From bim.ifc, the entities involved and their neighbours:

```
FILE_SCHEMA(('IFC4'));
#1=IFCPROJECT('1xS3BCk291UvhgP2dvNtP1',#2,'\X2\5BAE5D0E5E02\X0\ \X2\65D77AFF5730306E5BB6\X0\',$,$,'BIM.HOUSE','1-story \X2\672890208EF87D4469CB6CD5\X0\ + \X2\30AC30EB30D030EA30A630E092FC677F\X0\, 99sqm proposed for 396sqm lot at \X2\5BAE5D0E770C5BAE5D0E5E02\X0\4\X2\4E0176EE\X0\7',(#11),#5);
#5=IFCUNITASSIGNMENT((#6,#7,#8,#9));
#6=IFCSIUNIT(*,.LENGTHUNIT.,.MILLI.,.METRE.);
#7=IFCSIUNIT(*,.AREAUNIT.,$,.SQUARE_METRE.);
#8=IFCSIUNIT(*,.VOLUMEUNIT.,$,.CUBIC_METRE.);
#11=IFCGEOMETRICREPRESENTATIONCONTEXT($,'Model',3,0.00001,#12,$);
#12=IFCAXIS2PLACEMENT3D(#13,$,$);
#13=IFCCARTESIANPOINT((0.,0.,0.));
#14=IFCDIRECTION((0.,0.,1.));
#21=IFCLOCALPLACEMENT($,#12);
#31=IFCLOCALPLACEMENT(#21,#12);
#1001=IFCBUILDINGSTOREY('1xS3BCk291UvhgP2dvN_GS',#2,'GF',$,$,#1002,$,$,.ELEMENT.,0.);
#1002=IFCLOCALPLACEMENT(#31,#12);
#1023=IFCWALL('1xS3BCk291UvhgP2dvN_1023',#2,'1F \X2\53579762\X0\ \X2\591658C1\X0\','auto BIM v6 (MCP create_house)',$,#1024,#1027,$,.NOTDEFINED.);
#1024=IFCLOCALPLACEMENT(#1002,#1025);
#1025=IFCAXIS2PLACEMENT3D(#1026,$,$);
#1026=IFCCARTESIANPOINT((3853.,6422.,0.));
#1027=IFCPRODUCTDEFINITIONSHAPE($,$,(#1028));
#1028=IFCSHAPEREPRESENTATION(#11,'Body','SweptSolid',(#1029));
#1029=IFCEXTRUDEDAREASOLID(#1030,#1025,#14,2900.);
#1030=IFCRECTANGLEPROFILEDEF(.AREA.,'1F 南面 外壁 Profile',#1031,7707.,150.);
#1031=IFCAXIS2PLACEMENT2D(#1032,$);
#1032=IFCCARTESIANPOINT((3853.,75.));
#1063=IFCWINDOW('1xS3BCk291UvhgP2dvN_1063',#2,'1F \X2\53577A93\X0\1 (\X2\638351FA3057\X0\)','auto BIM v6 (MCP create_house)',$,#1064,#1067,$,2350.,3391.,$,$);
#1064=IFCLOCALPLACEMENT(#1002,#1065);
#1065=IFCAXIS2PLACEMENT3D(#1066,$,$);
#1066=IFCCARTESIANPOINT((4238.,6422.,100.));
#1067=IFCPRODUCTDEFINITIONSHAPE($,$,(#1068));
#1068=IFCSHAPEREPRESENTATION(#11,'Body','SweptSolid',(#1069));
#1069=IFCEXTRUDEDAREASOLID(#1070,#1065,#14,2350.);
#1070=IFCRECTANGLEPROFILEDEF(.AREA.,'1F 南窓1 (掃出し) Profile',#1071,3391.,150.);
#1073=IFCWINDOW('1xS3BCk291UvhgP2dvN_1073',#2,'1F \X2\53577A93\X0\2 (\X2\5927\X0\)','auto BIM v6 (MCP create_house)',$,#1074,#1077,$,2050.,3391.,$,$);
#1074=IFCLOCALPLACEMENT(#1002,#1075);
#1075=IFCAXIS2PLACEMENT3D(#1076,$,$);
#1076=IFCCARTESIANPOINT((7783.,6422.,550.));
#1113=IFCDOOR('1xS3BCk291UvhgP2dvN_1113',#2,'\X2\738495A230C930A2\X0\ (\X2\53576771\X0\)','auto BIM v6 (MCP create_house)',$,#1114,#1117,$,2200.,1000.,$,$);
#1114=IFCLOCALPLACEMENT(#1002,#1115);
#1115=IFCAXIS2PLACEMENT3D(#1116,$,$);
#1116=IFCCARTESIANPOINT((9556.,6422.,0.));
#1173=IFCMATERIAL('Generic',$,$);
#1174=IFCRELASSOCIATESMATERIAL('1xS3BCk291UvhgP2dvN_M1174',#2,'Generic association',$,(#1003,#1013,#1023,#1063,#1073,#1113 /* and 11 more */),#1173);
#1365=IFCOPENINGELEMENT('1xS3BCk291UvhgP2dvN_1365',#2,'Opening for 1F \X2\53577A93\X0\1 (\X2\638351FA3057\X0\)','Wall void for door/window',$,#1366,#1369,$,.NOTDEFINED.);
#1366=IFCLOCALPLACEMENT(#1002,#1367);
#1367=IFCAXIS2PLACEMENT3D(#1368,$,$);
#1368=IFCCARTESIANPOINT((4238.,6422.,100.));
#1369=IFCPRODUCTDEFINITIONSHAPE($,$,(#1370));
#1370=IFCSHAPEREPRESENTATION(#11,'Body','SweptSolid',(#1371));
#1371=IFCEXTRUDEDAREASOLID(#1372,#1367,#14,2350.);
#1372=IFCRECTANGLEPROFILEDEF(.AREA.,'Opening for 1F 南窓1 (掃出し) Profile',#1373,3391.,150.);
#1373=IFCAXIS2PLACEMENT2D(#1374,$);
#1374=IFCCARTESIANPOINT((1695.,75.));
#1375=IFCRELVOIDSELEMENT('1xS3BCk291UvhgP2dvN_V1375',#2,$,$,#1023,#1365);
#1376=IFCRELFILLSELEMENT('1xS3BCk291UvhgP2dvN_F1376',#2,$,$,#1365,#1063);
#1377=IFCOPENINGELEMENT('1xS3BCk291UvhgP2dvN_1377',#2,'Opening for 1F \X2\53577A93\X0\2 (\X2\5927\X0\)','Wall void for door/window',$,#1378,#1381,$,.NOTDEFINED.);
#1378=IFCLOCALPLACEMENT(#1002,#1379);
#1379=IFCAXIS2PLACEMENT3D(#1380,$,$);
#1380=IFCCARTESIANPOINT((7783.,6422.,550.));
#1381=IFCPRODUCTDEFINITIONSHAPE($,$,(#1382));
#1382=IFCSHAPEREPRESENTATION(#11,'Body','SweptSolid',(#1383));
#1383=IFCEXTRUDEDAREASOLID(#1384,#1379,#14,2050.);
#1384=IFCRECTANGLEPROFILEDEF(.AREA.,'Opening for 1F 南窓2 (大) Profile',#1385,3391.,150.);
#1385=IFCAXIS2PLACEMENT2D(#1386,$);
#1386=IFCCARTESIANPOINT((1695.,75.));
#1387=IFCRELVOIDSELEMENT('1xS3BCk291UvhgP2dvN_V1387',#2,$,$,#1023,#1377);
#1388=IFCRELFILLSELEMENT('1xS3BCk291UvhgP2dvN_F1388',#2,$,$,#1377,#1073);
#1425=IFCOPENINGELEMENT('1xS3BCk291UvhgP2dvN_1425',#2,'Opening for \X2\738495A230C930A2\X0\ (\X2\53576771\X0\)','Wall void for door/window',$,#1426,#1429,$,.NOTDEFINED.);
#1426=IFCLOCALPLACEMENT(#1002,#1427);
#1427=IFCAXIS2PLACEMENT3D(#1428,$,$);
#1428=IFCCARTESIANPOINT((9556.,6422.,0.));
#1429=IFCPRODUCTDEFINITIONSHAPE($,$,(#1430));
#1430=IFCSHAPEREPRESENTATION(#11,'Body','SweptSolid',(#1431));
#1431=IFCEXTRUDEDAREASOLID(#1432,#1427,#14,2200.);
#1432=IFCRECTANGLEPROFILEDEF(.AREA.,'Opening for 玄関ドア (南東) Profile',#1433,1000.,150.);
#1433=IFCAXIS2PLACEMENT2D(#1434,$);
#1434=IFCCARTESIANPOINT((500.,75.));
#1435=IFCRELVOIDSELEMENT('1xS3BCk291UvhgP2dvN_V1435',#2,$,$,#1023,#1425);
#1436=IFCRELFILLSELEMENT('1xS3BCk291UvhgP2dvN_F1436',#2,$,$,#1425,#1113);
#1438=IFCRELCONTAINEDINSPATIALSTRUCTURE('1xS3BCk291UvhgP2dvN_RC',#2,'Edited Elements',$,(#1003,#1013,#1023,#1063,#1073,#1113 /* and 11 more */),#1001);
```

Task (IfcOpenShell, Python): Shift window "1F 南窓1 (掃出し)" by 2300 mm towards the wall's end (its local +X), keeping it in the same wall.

```python
import ifcopenshell
import ifcopenshell.api.geometry
import ifcopenshell.util.placement
import ifcopenshell.util.unit

model = ifcopenshell.open("bim.ifc")
unit_scale = ifcopenshell.util.unit.calculate_unit_scale(model)

window = model.by_id(1063)
opening = window.FillsVoids[0].RelatingOpeningElement
wall = opening.VoidsElements[0].RelatingBuildingElement

wall_matrix = ifcopenshell.util.placement.get_local_placement(wall.ObjectPlacement)
shift = wall_matrix[:3, 0] * 2.3 / unit_scale
before = ifcopenshell.util.placement.get_local_placement(window.ObjectPlacement)[:3, 3].copy()

# The window is not placed relative to its opening, so move both.
for product in (opening, window):
    matrix = ifcopenshell.util.placement.get_local_placement(product.ObjectPlacement)
    matrix[:3, 3] += shift
    ifcopenshell.api.geometry.edit_object_placement(model, product=product, matrix=matrix, is_si=False)

after = ifcopenshell.util.placement.get_local_placement(window.ObjectPlacement)[:3, 3]
print("window moved by", (after - before).round(3) + 0.0)

model.write("bim_updated.ifc")
```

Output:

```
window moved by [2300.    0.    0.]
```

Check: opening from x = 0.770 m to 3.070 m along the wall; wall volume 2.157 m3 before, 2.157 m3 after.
